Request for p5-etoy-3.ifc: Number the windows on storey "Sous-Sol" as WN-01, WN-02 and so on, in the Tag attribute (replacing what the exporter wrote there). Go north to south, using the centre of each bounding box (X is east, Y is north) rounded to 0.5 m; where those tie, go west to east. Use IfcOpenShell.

First a look at what the model holds.

```python
import ifcopenshell
import ifcopenshell.util.element
import ifcopenshell.util.placement

model = ifcopenshell.open("p5-etoy-3.ifc")
print(model.schema)
storey = next(s for s in model.by_type("IfcBuildingStorey") if s.Name == "Sous-Sol")
windows = [e for e in ifcopenshell.util.element.get_decomposition(storey) if e.is_a("IfcWindow")]
for e in sorted(windows, key=lambda e: e.id()):
    origin = ifcopenshell.util.placement.get_local_placement(e.ObjectPlacement)[:3, 3]
    print(e.id(), e.Tag, e.Name, origin.round(2) + 0.0, sep=" | ")
```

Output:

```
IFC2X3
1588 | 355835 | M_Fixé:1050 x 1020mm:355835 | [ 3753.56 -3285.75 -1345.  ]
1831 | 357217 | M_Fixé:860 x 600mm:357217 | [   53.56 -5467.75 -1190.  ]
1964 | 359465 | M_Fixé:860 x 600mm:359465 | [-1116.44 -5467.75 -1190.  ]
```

```python
import ifcopenshell
import ifcopenshell.geom
import ifcopenshell.util.element
import ifcopenshell.util.shape

model = ifcopenshell.open("p5-etoy-3.ifc")
settings = ifcopenshell.geom.settings()
settings.set("use-world-coords", True)


def centre(element):
    shape = ifcopenshell.geom.create_shape(settings, element)
    return ifcopenshell.util.shape.get_bbox_centroid(shape.geometry)


storey = next(s for s in model.by_type("IfcBuildingStorey") if s.Name == "Sous-Sol")
windows = [e for e in ifcopenshell.util.element.get_decomposition(storey) if e.is_a("IfcWindow")]

# Insertion points can sit at a corner or the storey origin, so sort by the geometry (in metres).
centres = {e: centre(e) for e in windows}
windows.sort(key=lambda e: (-round(centres[e][1] / 0.5), centres[e][0]))

for i, e in enumerate(windows, start=1):
    number = f"WN-{i:02d}"
    e.Tag = number
    print(e.id(), number)

model.write("p5-etoy-3_rev.ifc")
```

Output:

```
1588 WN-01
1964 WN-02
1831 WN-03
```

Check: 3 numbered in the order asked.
